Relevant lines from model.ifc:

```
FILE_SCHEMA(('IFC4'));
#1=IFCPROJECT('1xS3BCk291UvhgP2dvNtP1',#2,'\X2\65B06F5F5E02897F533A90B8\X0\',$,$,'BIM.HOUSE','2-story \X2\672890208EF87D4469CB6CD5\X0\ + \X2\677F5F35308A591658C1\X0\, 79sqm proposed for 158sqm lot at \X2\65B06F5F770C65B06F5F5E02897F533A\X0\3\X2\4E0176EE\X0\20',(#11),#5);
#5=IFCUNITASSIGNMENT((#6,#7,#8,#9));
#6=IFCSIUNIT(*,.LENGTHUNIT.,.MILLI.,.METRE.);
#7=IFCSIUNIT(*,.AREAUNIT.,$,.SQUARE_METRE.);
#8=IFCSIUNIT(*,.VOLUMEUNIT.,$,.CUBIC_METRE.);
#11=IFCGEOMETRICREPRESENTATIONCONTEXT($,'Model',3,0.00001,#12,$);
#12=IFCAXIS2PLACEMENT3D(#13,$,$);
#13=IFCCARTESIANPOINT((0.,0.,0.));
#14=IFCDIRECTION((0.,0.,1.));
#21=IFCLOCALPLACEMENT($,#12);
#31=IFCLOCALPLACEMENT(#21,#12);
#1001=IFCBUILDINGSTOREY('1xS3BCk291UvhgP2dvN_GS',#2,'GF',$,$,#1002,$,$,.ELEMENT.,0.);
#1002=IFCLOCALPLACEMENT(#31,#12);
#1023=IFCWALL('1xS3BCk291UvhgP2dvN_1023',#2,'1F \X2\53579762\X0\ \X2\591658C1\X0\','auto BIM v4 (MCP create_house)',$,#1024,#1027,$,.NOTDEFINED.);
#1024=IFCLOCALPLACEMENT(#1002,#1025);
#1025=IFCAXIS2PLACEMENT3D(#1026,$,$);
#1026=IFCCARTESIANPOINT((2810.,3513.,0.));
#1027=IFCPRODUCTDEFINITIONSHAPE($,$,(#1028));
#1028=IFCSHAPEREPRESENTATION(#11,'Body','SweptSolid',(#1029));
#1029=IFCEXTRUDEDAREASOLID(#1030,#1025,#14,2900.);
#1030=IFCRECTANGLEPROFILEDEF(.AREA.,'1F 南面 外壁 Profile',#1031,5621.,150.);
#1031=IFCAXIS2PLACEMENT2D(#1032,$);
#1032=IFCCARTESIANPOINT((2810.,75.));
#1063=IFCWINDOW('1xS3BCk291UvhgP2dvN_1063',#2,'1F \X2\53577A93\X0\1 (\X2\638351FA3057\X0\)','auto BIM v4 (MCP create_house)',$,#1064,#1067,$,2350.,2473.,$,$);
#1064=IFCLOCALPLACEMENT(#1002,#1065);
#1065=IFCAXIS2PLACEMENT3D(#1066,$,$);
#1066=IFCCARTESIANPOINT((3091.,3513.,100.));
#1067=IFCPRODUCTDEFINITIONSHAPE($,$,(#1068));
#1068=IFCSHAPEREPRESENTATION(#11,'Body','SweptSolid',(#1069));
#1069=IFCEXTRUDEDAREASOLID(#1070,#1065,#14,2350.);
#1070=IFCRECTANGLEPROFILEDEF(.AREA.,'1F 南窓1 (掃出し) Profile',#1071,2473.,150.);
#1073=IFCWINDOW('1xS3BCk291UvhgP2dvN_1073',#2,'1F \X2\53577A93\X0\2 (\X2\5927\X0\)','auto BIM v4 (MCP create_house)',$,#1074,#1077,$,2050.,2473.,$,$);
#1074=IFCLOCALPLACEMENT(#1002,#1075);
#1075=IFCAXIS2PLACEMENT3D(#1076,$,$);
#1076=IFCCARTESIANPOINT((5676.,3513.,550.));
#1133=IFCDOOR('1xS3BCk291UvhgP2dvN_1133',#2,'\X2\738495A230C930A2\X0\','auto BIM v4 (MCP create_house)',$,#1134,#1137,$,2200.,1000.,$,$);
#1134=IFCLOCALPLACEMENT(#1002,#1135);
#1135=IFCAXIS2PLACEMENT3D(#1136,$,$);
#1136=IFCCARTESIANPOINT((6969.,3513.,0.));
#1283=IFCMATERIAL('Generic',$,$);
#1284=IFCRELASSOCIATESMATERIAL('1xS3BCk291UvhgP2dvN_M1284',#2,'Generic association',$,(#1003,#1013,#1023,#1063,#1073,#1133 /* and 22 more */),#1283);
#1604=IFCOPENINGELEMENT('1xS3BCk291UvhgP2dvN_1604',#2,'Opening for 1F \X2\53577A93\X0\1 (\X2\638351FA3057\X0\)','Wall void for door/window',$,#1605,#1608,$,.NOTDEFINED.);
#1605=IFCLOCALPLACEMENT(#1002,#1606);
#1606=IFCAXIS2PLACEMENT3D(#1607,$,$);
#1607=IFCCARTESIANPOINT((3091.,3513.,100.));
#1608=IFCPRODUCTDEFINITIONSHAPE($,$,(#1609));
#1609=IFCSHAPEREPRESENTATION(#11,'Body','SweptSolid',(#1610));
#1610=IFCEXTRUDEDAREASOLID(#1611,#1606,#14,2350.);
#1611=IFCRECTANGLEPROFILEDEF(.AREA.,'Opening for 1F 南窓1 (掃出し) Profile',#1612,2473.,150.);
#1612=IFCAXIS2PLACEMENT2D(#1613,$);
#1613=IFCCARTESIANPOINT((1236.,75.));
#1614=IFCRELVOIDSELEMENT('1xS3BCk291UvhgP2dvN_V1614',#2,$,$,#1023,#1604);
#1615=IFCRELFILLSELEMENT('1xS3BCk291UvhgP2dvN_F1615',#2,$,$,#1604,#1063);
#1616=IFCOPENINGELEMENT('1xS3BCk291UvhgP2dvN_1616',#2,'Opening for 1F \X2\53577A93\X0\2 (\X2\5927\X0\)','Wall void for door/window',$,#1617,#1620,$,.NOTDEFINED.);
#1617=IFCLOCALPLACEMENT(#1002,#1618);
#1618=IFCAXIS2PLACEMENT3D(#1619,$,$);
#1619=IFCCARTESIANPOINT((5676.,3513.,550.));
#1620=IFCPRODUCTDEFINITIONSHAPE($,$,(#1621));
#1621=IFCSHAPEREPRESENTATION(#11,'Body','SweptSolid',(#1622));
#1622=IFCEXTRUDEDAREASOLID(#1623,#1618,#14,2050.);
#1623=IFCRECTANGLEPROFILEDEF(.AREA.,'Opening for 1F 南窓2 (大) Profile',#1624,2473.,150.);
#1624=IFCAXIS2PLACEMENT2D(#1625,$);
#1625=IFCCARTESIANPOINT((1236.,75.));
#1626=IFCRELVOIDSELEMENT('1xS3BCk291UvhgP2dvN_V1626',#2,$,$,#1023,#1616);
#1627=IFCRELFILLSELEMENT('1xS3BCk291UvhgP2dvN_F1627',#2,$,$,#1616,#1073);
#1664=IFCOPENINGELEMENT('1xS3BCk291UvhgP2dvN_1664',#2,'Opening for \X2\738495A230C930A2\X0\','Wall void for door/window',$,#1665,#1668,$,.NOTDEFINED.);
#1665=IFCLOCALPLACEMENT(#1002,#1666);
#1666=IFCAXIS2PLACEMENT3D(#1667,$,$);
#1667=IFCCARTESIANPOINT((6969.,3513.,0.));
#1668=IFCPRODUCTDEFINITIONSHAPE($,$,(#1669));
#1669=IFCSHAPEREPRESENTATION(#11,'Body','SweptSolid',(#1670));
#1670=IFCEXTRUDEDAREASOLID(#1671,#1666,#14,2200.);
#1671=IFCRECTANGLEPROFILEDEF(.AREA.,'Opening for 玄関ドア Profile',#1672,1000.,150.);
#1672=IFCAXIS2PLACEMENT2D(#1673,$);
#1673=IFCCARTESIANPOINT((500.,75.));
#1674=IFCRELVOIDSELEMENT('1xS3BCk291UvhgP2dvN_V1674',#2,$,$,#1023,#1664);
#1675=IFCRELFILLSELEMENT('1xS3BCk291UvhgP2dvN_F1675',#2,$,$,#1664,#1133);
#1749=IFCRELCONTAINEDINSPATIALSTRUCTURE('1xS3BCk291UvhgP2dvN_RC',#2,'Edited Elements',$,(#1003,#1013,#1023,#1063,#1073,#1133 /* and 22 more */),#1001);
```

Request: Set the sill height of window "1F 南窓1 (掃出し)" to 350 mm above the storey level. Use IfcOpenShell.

```python
import numpy as np
import ifcopenshell
import ifcopenshell.api.geometry
import ifcopenshell.geom
import ifcopenshell.util.element
import ifcopenshell.util.placement
import ifcopenshell.util.shape
import ifcopenshell.util.unit

model = ifcopenshell.open("model.ifc")
unit_scale = ifcopenshell.util.unit.calculate_unit_scale(model)

window = model.by_guid("1xS3BCk291UvhgP2dvN_1063")
opening = window.FillsVoids[0].RelatingOpeningElement
storey = ifcopenshell.util.element.get_container(window, ifc_class="IfcBuildingStorey")
level = ifcopenshell.util.placement.get_local_placement(storey.ObjectPlacement)[2, 3]

# The opening's origin need not be at the sill, so measure its lowest point.
shape = ifcopenshell.geom.create_shape(ifcopenshell.geom.settings(), opening)
bottom = ifcopenshell.util.shape.get_shape_bottom_elevation(shape, shape.geometry) / unit_scale
dz = level + 350.0 - bottom

shift = np.array([0.0, 0.0, dz])
# The window is not placed relative to its opening, so move both.
for product in (opening, window):
    matrix = ifcopenshell.util.placement.get_local_placement(product.ObjectPlacement)
    matrix[:3, 3] += shift
    ifcopenshell.api.geometry.edit_object_placement(model, product=product, matrix=matrix, is_si=False)

print(f"moved by {dz * unit_scale:+.3f} m")

model.write("model_rev.ifc")
```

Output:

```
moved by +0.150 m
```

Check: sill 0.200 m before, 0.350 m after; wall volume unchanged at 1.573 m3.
